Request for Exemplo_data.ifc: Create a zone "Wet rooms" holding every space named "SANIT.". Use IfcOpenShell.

First a look at what the model holds.

```python
import ifcopenshell

model = ifcopenshell.open("Exemplo_data.ifc")
print(model.schema)
seen = {}
for space in model.by_type("IfcSpace"):
    seen[space.LongName] = seen.get(space.LongName, 0) + 1
for name, count in sorted(seen.items(), key=str):
    print(count, "x", name)
print("zones:", [z.Name for z in model.by_type("IfcZone")][:20])
```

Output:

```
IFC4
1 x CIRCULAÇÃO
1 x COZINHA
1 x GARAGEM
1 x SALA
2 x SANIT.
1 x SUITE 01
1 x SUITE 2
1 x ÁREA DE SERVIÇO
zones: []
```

```python
import ifcopenshell
import ifcopenshell.api.group
import ifcopenshell.api.root

model = ifcopenshell.open("Exemplo_data.ifc")

names = {"SANIT."}
spaces = [s for s in model.by_type("IfcSpace") if s.LongName in names]

zone = ifcopenshell.api.root.create_entity(model, ifc_class="IfcZone", name="Wet rooms")
ifcopenshell.api.group.assign_group(model, products=spaces, group=zone)
print(len(spaces), "spaces in", zone.Name)

model.write("Exemplo_data-out.ifc")
```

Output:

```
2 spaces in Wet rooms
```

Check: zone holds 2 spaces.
